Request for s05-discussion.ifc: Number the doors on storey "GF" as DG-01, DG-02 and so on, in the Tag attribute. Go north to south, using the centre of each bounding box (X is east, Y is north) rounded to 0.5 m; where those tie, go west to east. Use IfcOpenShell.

First a look at what the model holds.

```python
import ifcopenshell
import ifcopenshell.util.element
import ifcopenshell.util.placement

model = ifcopenshell.open("s05-discussion.ifc")
print(model.schema)
storey = next(s for s in model.by_type("IfcBuildingStorey") if s.Name == "GF")
doors = [e for e in ifcopenshell.util.element.get_decomposition(storey) if e.is_a("IfcDoor")]
for e in sorted(doors, key=lambda e: e.id()):
    origin = ifcopenshell.util.placement.get_local_placement(e.ObjectPlacement)[:3, 3]
    print(e.id(), e.Tag, e.Name, origin.round(2) + 0.0, sep=" | ")
```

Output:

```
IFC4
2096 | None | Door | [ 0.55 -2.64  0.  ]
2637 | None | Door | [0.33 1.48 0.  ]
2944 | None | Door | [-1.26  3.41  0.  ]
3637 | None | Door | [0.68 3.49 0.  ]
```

```python
import ifcopenshell
import ifcopenshell.geom
import ifcopenshell.util.element
import ifcopenshell.util.shape

model = ifcopenshell.open("s05-discussion.ifc")
settings = ifcopenshell.geom.settings()
settings.set("use-world-coords", True)


def centre(element):
    shape = ifcopenshell.geom.create_shape(settings, element)
    return ifcopenshell.util.shape.get_bbox_centroid(shape.geometry)


storey = next(s for s in model.by_type("IfcBuildingStorey") if s.Name == "GF")
doors = [e for e in ifcopenshell.util.element.get_decomposition(storey) if e.is_a("IfcDoor")]

# Insertion points can sit at a corner or the storey origin, so sort by the geometry (in metres).
centres = {e: centre(e) for e in doors}
doors.sort(key=lambda e: (-round(centres[e][1] / 0.5), centres[e][0]))

for i, e in enumerate(doors, start=1):
    number = f"DG-{i:02d}"
    e.Tag = number
    print(e.id(), number)

model.write("s05-discussion_edited.ifc")
```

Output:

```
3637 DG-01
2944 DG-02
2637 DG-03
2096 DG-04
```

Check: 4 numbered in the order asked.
